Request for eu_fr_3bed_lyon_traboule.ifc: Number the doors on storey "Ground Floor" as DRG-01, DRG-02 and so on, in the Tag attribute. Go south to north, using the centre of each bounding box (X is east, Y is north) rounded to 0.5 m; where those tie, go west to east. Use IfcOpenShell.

First a look at what the model holds.

```python
import ifcopenshell
import ifcopenshell.util.element
import ifcopenshell.util.placement

model = ifcopenshell.open("eu_fr_3bed_lyon_traboule.ifc")
print(model.schema)
storey = next(s for s in model.by_type("IfcBuildingStorey") if s.Name == "Ground Floor")
doors = [e for e in ifcopenshell.util.element.get_decomposition(storey) if e.is_a("IfcDoor")]
for e in sorted(doors, key=lambda e: e.id()):
    origin = ifcopenshell.util.placement.get_local_placement(e.ObjectPlacement)[:3, 3]
    print(e.id(), e.Tag, e.Name, origin.round(2) + 0.0, sep=" | ")
```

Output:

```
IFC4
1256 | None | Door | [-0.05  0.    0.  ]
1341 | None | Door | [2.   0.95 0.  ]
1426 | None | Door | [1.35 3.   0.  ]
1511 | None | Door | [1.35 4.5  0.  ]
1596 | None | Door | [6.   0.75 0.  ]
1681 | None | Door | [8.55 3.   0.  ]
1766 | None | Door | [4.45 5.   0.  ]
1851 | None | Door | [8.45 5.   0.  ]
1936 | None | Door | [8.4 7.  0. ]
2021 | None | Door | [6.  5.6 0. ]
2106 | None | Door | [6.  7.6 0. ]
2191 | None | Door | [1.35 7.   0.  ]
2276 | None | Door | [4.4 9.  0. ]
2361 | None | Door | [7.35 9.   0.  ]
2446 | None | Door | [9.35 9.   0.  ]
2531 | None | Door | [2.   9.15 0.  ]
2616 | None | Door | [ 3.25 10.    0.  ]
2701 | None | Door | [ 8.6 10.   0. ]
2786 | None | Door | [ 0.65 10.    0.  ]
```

```python
import ifcopenshell
import ifcopenshell.geom
import ifcopenshell.util.element
import ifcopenshell.util.shape

model = ifcopenshell.open("eu_fr_3bed_lyon_traboule.ifc")
settings = ifcopenshell.geom.settings()
settings.set("use-world-coords", True)


def centre(element):
    shape = ifcopenshell.geom.create_shape(settings, element)
    return ifcopenshell.util.shape.get_bbox_centroid(shape.geometry)


storey = next(s for s in model.by_type("IfcBuildingStorey") if s.Name == "Ground Floor")
doors = [e for e in ifcopenshell.util.element.get_decomposition(storey) if e.is_a("IfcDoor")]

# Insertion points can sit at a corner or the storey origin, so sort by the geometry (in metres).
centres = {e: centre(e) for e in doors}
doors.sort(key=lambda e: (round(centres[e][1] / 0.5), centres[e][0]))

for i, e in enumerate(doors, start=1):
    number = f"DRG-{i:02d}"
    e.Tag = number
    print(e.id(), number)

model.write("eu_fr_3bed_lyon_traboule_updated.ifc")
```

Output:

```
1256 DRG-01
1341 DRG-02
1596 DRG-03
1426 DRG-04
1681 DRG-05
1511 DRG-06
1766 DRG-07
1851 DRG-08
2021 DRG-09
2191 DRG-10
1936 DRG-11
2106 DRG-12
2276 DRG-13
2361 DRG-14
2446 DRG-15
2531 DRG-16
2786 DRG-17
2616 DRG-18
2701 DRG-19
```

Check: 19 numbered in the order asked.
